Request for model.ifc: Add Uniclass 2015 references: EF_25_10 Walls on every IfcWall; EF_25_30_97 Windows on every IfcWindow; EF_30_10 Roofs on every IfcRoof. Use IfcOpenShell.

First a look at what the model holds.

```python
import ifcopenshell

model = ifcopenshell.open("model.ifc")
print(model.schema)
print("classifications:", [c.Name for c in model.by_type("IfcClassification")])
for ifc_class in ("IfcDoor", "IfcRoof", "IfcStair", "IfcWall", "IfcWindow"):
    print(ifc_class, len(model.by_type(ifc_class)))
```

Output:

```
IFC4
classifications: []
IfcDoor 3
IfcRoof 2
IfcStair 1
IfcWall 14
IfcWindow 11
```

```python
import ifcopenshell
import ifcopenshell.api.classification

model = ifcopenshell.open("model.ifc")

system = ifcopenshell.api.classification.add_classification(model, classification="Uniclass 2015")

codes = {
    "IfcWall": ("EF_25_10", "Walls"),
    "IfcWindow": ("EF_25_30_97", "Windows"),
    "IfcRoof": ("EF_30_10", "Roofs"),
}
for ifc_class, (code, name) in codes.items():
    products = model.by_type(ifc_class)
    ifcopenshell.api.classification.add_reference(
        model, products=products, classification=system, identification=code, name=name
    )
    print(code, len(products))

model.write("model-out.ifc")
```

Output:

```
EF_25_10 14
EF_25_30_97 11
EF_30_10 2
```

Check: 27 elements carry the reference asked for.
